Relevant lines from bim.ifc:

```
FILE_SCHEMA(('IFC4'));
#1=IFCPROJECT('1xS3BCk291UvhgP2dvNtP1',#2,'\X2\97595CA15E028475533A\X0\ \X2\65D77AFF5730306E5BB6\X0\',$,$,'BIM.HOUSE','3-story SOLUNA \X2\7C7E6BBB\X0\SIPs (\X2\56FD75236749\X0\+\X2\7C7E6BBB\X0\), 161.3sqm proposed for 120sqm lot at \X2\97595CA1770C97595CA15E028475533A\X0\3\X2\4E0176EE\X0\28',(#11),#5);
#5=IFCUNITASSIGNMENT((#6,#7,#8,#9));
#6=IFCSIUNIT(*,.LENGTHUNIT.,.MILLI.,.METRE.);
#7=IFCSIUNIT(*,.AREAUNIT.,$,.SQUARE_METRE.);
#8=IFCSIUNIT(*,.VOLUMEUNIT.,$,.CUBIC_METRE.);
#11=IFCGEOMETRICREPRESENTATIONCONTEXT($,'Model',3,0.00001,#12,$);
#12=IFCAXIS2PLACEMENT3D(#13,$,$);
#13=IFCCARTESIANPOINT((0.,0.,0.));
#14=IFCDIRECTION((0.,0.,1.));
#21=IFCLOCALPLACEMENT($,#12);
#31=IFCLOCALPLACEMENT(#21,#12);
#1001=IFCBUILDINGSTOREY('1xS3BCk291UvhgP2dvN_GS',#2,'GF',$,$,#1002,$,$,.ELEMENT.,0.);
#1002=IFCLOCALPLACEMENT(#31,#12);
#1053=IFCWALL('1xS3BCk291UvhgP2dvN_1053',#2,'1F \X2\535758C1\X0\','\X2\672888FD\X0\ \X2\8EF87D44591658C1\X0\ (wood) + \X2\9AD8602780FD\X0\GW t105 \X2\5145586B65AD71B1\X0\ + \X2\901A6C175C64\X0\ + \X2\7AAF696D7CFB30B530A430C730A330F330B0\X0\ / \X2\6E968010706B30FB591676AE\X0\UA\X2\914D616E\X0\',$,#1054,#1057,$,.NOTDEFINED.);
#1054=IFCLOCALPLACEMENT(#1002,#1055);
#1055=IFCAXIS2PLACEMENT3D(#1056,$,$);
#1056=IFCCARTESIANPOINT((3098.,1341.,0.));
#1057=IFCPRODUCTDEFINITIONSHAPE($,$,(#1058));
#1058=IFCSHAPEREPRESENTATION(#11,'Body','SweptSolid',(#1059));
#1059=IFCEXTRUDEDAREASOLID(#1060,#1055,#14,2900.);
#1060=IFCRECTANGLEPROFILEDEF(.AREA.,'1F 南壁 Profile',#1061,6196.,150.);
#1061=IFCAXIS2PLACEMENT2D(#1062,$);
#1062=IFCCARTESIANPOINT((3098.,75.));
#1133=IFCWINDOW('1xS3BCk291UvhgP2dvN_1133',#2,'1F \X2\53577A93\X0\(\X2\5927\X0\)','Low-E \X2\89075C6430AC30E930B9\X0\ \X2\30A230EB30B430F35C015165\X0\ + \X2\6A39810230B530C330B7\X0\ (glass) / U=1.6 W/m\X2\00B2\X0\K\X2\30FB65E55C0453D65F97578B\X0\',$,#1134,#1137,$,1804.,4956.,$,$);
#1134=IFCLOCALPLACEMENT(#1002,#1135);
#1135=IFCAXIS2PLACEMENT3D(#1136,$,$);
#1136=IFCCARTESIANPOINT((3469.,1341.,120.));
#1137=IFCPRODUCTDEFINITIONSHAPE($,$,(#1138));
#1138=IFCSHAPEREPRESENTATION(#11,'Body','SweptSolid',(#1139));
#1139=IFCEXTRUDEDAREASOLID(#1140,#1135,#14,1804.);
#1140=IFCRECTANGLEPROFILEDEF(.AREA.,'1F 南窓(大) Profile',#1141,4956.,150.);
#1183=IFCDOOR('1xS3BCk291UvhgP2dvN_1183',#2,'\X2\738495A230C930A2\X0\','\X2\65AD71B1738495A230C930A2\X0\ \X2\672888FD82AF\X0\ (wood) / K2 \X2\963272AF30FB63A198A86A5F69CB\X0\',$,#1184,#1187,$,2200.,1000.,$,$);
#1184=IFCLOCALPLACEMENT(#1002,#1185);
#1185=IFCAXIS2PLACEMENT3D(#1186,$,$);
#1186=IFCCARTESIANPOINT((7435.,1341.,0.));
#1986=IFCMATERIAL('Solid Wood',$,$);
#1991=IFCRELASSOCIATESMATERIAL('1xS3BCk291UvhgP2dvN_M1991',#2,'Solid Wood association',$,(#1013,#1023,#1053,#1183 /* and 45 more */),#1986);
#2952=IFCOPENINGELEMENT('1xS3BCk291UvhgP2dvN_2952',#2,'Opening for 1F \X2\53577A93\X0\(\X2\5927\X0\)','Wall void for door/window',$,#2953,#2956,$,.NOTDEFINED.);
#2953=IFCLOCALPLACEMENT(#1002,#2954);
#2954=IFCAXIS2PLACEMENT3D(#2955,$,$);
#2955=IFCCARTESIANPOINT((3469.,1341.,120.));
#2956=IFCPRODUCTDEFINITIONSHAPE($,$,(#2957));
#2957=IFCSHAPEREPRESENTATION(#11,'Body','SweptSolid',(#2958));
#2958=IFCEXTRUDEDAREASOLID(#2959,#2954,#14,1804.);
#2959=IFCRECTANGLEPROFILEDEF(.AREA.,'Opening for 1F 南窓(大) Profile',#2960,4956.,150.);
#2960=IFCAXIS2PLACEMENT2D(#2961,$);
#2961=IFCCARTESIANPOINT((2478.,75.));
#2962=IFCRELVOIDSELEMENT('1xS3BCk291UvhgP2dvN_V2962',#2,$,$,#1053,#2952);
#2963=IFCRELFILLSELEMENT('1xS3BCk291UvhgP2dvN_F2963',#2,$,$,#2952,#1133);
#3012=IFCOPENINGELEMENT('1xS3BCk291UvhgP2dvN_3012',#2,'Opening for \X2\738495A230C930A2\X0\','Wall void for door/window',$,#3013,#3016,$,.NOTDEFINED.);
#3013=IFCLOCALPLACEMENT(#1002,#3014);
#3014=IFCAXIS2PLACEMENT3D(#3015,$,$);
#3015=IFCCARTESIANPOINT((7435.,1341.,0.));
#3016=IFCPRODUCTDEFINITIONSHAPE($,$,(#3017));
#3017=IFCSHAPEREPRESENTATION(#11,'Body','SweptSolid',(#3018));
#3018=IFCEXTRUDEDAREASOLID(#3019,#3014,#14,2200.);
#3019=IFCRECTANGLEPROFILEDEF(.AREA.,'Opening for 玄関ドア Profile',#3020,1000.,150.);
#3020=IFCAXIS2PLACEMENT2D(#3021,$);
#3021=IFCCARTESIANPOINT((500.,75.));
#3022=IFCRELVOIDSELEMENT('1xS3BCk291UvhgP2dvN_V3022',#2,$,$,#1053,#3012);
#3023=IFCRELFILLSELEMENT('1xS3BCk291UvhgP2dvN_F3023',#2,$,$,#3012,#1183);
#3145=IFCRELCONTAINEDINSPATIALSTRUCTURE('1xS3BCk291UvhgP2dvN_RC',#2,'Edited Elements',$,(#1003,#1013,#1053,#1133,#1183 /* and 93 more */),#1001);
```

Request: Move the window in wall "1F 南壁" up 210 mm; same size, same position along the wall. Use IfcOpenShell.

```python
import numpy as np
import ifcopenshell
import ifcopenshell.api.geometry
import ifcopenshell.util.placement
import ifcopenshell.util.unit

model = ifcopenshell.open("bim.ifc")
unit_scale = ifcopenshell.util.unit.calculate_unit_scale(model)

window = model.by_id(1133)
opening = window.FillsVoids[0].RelatingOpeningElement
dz = 0.21 / unit_scale

shift = np.array([0.0, 0.0, dz])
# The window is not placed relative to its opening, so move both.
for product in (opening, window):
    matrix = ifcopenshell.util.placement.get_local_placement(product.ObjectPlacement)
    matrix[:3, 3] += shift
    ifcopenshell.api.geometry.edit_object_placement(model, product=product, matrix=matrix, is_si=False)

print(f"moved by {dz * unit_scale:+.3f} m")

model.write("bim-out.ifc")
```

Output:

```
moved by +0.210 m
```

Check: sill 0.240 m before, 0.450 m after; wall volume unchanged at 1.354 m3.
